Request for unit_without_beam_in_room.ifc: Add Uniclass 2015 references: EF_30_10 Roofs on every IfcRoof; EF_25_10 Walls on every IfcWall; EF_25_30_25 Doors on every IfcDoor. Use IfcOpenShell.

First a look at what the model holds.

```python
import ifcopenshell

model = ifcopenshell.open("unit_without_beam_in_room.ifc")
print(model.schema)
print("classifications:", [c.Name for c in model.by_type("IfcClassification")])
for ifc_class in ("IfcDoor", "IfcRoof", "IfcStair", "IfcWall", "IfcWindow"):
    print(ifc_class, len(model.by_type(ifc_class)))
```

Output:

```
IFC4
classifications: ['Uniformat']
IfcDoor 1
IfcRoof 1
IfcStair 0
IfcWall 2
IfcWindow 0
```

```python
import ifcopenshell
import ifcopenshell.api.classification

model = ifcopenshell.open("unit_without_beam_in_room.ifc")

system = ifcopenshell.api.classification.add_classification(model, classification="Uniclass 2015")

codes = {
    "IfcRoof": ("EF_30_10", "Roofs"),
    "IfcWall": ("EF_25_10", "Walls"),
    "IfcDoor": ("EF_25_30_25", "Doors"),
}
for ifc_class, (code, name) in codes.items():
    products = model.by_type(ifc_class)
    ifcopenshell.api.classification.add_reference(
        model, products=products, classification=system, identification=code, name=name
    )
    print(code, len(products))

model.write("unit_without_beam_in_room-out.ifc")
```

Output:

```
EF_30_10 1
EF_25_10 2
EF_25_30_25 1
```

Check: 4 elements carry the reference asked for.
